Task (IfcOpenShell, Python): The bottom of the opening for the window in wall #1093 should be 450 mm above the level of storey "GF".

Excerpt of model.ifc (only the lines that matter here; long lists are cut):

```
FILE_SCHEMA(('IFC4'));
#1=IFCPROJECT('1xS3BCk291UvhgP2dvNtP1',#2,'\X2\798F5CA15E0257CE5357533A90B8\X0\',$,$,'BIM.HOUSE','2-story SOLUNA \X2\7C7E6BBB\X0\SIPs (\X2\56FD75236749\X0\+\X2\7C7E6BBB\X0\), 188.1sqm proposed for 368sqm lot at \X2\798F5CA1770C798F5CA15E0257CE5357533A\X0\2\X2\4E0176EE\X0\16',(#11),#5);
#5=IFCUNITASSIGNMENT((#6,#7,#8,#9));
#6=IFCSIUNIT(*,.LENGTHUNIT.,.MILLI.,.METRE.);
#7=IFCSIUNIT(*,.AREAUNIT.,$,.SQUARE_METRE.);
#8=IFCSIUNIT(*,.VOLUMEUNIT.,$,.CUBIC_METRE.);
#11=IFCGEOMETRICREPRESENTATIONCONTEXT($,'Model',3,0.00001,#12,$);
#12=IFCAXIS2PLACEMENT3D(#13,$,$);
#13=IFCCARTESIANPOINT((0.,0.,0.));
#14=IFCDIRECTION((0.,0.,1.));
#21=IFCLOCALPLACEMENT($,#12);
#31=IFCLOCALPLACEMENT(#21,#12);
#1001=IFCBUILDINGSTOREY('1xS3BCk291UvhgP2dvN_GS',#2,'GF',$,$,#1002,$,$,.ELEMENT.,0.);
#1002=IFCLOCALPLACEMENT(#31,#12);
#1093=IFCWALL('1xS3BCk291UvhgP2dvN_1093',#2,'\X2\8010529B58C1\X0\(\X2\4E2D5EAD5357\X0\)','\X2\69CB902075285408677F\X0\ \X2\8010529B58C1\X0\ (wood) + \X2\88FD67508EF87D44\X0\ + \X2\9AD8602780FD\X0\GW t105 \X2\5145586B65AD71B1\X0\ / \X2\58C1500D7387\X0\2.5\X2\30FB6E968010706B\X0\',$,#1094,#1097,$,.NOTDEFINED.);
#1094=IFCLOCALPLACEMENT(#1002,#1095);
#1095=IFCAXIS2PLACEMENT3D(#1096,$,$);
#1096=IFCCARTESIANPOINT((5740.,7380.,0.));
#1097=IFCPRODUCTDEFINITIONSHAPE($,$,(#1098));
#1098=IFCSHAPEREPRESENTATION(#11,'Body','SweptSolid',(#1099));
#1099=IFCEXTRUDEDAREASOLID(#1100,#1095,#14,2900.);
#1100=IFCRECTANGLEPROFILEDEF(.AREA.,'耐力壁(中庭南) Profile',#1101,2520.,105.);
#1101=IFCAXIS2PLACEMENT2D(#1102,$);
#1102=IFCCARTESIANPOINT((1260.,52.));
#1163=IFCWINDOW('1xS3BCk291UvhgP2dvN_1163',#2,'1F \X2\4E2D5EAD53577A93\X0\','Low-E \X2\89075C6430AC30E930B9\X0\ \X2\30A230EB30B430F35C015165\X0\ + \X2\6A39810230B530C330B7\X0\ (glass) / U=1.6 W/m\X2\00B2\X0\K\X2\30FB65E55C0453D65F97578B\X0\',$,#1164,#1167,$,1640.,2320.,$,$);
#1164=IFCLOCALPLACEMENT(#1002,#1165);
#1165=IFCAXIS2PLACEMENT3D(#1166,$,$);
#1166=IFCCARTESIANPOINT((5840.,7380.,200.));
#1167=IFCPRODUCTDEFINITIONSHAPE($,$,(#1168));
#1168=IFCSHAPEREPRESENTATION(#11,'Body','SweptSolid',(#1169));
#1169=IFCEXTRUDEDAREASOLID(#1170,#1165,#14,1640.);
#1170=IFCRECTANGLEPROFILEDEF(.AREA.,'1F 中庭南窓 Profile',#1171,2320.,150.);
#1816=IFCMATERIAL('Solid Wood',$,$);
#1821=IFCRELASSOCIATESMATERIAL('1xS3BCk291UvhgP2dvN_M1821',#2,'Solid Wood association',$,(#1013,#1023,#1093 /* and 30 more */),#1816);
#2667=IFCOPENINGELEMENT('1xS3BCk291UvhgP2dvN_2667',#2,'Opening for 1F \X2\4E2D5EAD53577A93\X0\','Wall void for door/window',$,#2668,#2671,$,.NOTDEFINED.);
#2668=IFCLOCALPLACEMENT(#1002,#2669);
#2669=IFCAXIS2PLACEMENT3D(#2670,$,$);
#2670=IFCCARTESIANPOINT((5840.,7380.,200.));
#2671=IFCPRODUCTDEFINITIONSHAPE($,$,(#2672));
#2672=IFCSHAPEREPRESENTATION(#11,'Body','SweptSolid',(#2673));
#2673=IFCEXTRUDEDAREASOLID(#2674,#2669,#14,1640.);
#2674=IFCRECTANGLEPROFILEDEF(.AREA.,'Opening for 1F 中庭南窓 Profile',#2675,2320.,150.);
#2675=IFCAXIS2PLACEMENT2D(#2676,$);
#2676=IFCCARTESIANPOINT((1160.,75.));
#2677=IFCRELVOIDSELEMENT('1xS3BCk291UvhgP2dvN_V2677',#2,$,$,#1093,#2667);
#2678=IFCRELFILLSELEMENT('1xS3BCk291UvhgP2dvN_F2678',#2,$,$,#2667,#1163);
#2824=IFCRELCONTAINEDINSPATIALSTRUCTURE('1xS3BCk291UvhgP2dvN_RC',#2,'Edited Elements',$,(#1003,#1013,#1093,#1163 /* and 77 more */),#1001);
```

```python
import numpy as np
import ifcopenshell
import ifcopenshell.api.geometry
import ifcopenshell.geom
import ifcopenshell.util.element
import ifcopenshell.util.placement
import ifcopenshell.util.shape
import ifcopenshell.util.unit

model = ifcopenshell.open("model.ifc")
unit_scale = ifcopenshell.util.unit.calculate_unit_scale(model)

window = model.by_guid("1xS3BCk291UvhgP2dvN_1163")
opening = window.FillsVoids[0].RelatingOpeningElement
storey = ifcopenshell.util.element.get_container(window, ifc_class="IfcBuildingStorey")
level = ifcopenshell.util.placement.get_local_placement(storey.ObjectPlacement)[2, 3]

# The opening's origin need not be at the sill, so measure its lowest point.
shape = ifcopenshell.geom.create_shape(ifcopenshell.geom.settings(), opening)
bottom = ifcopenshell.util.shape.get_shape_bottom_elevation(shape, shape.geometry) / unit_scale
dz = level + 0.45 / unit_scale - bottom

shift = np.array([0.0, 0.0, dz])
# The window is not placed relative to its opening, so move both.
for product in (opening, window):
    matrix = ifcopenshell.util.placement.get_local_placement(product.ObjectPlacement)
    matrix[:3, 3] += shift
    ifcopenshell.api.geometry.edit_object_placement(model, product=product, matrix=matrix, is_si=False)

print(f"moved by {dz * unit_scale:+.3f} m")

model.write("model_updated.ifc")
```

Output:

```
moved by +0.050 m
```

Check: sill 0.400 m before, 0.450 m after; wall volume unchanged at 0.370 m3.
